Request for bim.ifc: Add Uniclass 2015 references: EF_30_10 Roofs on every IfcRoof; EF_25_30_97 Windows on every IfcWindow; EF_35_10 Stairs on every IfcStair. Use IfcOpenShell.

First a look at what the model holds.

```python
import ifcopenshell

model = ifcopenshell.open("bim.ifc")
print(model.schema)
print("classifications:", [c.Name for c in model.by_type("IfcClassification")])
for ifc_class in ("IfcDoor", "IfcRoof", "IfcStair", "IfcWall", "IfcWindow"):
    print(ifc_class, len(model.by_type(ifc_class)))
```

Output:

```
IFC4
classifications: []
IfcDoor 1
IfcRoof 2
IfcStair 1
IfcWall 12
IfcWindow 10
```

```python
import ifcopenshell
import ifcopenshell.api.classification

model = ifcopenshell.open("bim.ifc")

system = ifcopenshell.api.classification.add_classification(model, classification="Uniclass 2015")

codes = {
    "IfcRoof": ("EF_30_10", "Roofs"),
    "IfcWindow": ("EF_25_30_97", "Windows"),
    "IfcStair": ("EF_35_10", "Stairs"),
}
for ifc_class, (code, name) in codes.items():
    products = model.by_type(ifc_class)
    ifcopenshell.api.classification.add_reference(
        model, products=products, classification=system, identification=code, name=name
    )
    print(code, len(products))

model.write("bim_edited.ifc")
```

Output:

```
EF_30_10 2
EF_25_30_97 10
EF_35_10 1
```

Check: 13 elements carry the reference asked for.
